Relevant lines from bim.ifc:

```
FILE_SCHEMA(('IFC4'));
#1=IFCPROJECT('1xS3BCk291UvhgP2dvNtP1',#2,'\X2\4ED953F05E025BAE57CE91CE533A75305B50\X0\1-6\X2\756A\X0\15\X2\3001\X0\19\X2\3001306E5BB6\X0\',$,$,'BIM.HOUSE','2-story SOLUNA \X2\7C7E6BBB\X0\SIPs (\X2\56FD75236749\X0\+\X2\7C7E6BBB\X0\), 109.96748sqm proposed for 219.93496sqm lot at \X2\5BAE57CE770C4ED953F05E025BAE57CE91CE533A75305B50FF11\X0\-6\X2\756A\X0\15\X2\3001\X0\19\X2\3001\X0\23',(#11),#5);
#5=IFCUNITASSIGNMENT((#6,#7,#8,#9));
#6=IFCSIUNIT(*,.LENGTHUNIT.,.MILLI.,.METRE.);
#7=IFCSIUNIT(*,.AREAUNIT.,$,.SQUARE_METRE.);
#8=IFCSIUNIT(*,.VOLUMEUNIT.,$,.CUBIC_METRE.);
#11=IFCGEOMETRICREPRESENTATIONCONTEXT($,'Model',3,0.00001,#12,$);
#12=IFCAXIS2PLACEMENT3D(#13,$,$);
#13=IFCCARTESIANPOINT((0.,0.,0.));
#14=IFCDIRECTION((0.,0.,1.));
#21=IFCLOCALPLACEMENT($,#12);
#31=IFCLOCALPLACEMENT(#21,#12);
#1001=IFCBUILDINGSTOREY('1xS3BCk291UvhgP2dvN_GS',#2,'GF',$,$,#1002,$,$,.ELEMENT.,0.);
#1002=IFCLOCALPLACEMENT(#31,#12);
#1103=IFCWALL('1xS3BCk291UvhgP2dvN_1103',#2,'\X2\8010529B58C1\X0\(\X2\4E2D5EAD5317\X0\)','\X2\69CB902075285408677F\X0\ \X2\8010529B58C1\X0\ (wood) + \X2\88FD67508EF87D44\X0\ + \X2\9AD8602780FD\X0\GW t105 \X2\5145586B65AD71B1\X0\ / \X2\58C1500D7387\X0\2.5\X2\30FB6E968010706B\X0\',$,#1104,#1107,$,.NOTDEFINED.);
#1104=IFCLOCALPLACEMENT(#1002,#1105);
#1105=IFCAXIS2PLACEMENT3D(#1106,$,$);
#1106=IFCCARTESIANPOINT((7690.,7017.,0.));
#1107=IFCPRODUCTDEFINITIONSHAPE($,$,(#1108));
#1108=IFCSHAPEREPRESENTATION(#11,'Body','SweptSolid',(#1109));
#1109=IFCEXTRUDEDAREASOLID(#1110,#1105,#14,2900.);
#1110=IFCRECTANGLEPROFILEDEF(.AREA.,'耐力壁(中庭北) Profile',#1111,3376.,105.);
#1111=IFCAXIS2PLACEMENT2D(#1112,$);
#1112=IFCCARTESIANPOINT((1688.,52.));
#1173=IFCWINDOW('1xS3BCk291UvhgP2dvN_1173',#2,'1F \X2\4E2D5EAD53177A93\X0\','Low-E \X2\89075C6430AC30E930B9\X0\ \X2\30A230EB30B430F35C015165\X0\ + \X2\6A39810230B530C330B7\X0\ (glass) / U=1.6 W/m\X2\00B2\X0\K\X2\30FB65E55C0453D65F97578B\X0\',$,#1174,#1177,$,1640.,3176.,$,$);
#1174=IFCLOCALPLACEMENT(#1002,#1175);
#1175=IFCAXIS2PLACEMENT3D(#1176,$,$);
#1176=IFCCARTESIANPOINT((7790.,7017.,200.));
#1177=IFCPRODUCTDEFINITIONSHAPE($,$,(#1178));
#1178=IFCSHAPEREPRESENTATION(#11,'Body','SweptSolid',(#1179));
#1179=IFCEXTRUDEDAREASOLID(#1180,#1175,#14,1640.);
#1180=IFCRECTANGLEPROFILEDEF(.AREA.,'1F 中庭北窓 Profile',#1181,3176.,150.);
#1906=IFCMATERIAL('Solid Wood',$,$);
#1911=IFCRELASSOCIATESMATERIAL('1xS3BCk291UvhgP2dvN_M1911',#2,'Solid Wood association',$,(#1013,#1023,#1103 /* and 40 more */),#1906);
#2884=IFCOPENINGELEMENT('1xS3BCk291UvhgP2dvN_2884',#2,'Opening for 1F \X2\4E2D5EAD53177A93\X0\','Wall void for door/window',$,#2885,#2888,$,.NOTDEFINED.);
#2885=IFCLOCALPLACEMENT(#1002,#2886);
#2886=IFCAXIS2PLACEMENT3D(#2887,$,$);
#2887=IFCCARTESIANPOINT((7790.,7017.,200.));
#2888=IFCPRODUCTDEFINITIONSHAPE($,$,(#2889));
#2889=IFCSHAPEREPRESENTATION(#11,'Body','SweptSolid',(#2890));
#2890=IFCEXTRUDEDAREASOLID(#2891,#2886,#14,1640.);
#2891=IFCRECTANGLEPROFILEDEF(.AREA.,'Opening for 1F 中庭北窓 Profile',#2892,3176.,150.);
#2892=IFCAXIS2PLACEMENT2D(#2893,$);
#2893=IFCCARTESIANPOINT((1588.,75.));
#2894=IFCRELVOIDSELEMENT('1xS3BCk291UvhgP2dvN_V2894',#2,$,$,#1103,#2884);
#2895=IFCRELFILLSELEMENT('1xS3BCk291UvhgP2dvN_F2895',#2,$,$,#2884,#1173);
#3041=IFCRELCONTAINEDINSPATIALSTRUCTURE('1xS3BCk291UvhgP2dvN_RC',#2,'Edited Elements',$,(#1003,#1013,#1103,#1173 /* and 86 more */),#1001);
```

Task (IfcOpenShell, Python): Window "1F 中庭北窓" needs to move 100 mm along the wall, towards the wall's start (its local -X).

```python
import ifcopenshell
import ifcopenshell.api.geometry
import ifcopenshell.util.placement

model = ifcopenshell.open("bim.ifc")

window = model.by_guid("1xS3BCk291UvhgP2dvN_1173")
opening = window.FillsVoids[0].RelatingOpeningElement
wall = opening.VoidsElements[0].RelatingBuildingElement

wall_matrix = ifcopenshell.util.placement.get_local_placement(wall.ObjectPlacement)
shift = wall_matrix[:3, 0] * -100.0
before = ifcopenshell.util.placement.get_local_placement(window.ObjectPlacement)[:3, 3].copy()

# The window is not placed relative to its opening, so move both.
for product in (opening, window):
    matrix = ifcopenshell.util.placement.get_local_placement(product.ObjectPlacement)
    matrix[:3, 3] += shift
    ifcopenshell.api.geometry.edit_object_placement(model, product=product, matrix=matrix, is_si=False)

after = ifcopenshell.util.placement.get_local_placement(window.ObjectPlacement)[:3, 3]
print("window moved by", (after - before).round(3) + 0.0)

model.write("bim_edited.ifc")
```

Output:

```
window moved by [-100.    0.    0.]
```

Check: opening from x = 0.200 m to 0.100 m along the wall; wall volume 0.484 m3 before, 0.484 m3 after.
